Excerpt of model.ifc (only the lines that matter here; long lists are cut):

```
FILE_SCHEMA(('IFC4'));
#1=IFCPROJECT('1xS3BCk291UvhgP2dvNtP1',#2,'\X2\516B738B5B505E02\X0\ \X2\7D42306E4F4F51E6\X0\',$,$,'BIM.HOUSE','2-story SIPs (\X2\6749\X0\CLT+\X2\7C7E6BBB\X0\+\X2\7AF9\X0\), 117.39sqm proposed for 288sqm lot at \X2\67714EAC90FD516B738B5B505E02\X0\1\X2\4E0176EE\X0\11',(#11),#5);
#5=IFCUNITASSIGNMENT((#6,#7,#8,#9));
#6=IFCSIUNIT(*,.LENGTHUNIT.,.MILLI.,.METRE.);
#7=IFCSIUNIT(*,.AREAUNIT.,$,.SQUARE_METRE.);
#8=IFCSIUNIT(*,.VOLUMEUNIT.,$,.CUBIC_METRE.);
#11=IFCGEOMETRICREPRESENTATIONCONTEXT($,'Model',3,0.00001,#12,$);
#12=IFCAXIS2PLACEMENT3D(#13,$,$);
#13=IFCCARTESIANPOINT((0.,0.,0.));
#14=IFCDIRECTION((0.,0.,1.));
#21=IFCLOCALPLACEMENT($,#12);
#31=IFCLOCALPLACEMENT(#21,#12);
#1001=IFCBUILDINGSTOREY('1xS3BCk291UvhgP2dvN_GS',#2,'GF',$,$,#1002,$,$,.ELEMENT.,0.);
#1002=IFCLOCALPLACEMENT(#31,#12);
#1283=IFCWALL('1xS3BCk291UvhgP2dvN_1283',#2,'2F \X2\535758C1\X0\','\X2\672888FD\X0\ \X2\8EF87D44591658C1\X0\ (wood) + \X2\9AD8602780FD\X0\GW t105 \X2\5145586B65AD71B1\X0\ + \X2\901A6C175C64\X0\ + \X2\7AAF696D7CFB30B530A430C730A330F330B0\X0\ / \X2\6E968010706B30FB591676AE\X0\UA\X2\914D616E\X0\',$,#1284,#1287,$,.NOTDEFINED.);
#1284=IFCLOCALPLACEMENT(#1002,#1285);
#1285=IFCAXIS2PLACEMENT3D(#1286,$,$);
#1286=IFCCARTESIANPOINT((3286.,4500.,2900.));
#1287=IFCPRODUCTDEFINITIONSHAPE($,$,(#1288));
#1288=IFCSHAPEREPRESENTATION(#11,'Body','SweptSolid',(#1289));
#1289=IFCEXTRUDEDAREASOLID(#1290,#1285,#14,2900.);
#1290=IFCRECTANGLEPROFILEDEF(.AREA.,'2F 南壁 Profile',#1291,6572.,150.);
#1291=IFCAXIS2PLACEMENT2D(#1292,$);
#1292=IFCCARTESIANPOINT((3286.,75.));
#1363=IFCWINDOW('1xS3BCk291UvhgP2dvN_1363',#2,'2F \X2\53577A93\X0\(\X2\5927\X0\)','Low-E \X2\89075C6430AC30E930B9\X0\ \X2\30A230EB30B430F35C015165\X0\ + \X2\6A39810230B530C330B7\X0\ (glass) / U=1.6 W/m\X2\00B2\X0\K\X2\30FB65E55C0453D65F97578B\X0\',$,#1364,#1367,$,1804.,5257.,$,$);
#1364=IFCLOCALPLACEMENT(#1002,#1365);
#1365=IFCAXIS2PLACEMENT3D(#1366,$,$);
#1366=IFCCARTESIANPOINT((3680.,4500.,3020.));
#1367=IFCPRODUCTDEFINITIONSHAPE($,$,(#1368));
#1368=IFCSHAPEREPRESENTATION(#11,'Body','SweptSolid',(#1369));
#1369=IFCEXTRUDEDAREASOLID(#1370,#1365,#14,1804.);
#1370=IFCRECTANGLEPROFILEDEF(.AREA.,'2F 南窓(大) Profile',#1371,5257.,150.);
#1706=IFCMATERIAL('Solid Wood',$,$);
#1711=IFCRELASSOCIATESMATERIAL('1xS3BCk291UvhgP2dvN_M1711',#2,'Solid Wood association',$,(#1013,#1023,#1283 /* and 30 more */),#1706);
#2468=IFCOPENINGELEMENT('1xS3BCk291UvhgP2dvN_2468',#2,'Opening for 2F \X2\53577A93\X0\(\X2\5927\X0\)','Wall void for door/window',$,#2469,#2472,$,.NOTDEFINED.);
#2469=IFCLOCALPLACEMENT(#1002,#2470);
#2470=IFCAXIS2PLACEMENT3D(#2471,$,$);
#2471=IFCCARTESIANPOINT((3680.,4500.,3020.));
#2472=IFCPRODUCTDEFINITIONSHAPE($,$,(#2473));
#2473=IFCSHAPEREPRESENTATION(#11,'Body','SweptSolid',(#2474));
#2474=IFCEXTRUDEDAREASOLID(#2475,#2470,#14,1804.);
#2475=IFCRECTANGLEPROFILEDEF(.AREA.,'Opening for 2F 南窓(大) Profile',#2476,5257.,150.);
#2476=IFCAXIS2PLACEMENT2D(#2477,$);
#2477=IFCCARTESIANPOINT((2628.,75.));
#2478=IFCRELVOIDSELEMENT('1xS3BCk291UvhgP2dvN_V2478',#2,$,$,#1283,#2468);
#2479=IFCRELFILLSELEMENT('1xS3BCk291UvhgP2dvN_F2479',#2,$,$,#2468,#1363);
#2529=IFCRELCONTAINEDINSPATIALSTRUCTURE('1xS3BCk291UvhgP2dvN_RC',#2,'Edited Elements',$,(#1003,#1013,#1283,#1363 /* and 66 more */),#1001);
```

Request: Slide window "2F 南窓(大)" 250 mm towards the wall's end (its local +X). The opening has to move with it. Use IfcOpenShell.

```python
import ifcopenshell
import ifcopenshell.api.geometry
import ifcopenshell.util.placement

model = ifcopenshell.open("model.ifc")

window = model.by_id(1363)
opening = window.FillsVoids[0].RelatingOpeningElement
wall = opening.VoidsElements[0].RelatingBuildingElement

wall_matrix = ifcopenshell.util.placement.get_local_placement(wall.ObjectPlacement)
shift = wall_matrix[:3, 0] * 250.0
before = ifcopenshell.util.placement.get_local_placement(window.ObjectPlacement)[:3, 3].copy()

# The window is not placed relative to its opening, so move both.
for product in (opening, window):
    matrix = ifcopenshell.util.placement.get_local_placement(product.ObjectPlacement)
    matrix[:3, 3] += shift
    ifcopenshell.api.geometry.edit_object_placement(model, product=product, matrix=matrix, is_si=False)

after = ifcopenshell.util.placement.get_local_placement(window.ObjectPlacement)[:3, 3]
print("window moved by", (after - before).round(3) + 0.0)

model.write("model_v2.ifc")
```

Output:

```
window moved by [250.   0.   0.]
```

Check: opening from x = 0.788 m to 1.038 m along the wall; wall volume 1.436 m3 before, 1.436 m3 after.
